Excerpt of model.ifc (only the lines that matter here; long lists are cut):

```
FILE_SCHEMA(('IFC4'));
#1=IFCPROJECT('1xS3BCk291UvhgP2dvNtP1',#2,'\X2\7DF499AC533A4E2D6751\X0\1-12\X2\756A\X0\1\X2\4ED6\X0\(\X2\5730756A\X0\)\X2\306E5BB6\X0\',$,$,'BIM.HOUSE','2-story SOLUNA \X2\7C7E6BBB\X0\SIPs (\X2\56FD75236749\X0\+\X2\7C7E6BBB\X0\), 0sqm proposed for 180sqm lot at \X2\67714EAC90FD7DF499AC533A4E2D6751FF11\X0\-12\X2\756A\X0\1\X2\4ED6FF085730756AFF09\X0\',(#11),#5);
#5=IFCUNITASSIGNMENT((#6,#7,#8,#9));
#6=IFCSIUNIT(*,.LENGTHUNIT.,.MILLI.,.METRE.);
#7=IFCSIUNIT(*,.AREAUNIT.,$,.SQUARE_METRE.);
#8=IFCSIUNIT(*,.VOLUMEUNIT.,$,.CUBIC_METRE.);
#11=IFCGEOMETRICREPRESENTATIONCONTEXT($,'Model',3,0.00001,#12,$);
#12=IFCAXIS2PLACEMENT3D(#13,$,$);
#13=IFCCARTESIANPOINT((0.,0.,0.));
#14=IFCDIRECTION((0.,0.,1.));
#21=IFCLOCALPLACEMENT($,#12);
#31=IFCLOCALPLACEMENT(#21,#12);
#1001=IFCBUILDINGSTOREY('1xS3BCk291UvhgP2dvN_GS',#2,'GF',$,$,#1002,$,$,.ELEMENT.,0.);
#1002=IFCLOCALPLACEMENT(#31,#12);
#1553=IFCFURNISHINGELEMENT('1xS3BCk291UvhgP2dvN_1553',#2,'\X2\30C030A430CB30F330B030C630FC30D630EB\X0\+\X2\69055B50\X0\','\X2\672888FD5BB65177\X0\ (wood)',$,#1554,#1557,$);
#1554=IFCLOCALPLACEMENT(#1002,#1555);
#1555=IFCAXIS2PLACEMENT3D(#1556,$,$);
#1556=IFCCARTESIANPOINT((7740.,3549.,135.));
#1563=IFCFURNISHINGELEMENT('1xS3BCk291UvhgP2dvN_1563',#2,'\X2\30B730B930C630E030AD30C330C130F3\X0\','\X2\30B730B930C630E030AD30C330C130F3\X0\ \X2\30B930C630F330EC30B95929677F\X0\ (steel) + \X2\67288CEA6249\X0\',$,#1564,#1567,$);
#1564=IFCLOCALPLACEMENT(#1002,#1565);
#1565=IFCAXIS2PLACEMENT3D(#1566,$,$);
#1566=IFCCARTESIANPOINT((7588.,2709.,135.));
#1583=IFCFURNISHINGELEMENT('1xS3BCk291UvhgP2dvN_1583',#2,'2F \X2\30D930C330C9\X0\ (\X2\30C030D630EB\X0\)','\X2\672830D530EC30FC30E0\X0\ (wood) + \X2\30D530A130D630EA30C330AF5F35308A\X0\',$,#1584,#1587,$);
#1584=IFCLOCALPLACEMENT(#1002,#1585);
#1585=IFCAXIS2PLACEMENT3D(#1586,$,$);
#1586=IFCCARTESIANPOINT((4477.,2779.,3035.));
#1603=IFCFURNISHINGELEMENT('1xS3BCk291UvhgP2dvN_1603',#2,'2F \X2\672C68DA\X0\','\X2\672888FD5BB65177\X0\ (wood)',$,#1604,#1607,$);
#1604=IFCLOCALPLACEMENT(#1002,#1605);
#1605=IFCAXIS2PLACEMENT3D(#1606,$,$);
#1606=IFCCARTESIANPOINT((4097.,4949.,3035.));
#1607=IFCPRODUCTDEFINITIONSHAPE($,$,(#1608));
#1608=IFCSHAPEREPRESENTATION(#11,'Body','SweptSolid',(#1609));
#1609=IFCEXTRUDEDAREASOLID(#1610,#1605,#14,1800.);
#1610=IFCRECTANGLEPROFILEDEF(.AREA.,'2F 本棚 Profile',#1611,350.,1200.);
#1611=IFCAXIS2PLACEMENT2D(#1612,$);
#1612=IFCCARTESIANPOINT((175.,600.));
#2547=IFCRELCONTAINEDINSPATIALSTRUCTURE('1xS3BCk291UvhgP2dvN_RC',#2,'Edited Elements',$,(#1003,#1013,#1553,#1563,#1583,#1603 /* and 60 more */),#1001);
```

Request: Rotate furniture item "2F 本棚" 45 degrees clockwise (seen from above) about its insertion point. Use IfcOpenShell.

```python
import ifcopenshell
import ifcopenshell.api.geometry
import ifcopenshell.util.placement

model = ifcopenshell.open("model.ifc")

item = model.by_id(1603)
matrix = ifcopenshell.util.placement.get_local_placement(item.ObjectPlacement)
matrix = matrix @ ifcopenshell.util.placement.rotation(-45, "Z")
ifcopenshell.api.geometry.edit_object_placement(model, product=item, matrix=matrix, is_si=False)

print(ifcopenshell.util.placement.get_local_placement(item.ObjectPlacement).round(3) + 0.0)

model.write("model_updated.ifc")
```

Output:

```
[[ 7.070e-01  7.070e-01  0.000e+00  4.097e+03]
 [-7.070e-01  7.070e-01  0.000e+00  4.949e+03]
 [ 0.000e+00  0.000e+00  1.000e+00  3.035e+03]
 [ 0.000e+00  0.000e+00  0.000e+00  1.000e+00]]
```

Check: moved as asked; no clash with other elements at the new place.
